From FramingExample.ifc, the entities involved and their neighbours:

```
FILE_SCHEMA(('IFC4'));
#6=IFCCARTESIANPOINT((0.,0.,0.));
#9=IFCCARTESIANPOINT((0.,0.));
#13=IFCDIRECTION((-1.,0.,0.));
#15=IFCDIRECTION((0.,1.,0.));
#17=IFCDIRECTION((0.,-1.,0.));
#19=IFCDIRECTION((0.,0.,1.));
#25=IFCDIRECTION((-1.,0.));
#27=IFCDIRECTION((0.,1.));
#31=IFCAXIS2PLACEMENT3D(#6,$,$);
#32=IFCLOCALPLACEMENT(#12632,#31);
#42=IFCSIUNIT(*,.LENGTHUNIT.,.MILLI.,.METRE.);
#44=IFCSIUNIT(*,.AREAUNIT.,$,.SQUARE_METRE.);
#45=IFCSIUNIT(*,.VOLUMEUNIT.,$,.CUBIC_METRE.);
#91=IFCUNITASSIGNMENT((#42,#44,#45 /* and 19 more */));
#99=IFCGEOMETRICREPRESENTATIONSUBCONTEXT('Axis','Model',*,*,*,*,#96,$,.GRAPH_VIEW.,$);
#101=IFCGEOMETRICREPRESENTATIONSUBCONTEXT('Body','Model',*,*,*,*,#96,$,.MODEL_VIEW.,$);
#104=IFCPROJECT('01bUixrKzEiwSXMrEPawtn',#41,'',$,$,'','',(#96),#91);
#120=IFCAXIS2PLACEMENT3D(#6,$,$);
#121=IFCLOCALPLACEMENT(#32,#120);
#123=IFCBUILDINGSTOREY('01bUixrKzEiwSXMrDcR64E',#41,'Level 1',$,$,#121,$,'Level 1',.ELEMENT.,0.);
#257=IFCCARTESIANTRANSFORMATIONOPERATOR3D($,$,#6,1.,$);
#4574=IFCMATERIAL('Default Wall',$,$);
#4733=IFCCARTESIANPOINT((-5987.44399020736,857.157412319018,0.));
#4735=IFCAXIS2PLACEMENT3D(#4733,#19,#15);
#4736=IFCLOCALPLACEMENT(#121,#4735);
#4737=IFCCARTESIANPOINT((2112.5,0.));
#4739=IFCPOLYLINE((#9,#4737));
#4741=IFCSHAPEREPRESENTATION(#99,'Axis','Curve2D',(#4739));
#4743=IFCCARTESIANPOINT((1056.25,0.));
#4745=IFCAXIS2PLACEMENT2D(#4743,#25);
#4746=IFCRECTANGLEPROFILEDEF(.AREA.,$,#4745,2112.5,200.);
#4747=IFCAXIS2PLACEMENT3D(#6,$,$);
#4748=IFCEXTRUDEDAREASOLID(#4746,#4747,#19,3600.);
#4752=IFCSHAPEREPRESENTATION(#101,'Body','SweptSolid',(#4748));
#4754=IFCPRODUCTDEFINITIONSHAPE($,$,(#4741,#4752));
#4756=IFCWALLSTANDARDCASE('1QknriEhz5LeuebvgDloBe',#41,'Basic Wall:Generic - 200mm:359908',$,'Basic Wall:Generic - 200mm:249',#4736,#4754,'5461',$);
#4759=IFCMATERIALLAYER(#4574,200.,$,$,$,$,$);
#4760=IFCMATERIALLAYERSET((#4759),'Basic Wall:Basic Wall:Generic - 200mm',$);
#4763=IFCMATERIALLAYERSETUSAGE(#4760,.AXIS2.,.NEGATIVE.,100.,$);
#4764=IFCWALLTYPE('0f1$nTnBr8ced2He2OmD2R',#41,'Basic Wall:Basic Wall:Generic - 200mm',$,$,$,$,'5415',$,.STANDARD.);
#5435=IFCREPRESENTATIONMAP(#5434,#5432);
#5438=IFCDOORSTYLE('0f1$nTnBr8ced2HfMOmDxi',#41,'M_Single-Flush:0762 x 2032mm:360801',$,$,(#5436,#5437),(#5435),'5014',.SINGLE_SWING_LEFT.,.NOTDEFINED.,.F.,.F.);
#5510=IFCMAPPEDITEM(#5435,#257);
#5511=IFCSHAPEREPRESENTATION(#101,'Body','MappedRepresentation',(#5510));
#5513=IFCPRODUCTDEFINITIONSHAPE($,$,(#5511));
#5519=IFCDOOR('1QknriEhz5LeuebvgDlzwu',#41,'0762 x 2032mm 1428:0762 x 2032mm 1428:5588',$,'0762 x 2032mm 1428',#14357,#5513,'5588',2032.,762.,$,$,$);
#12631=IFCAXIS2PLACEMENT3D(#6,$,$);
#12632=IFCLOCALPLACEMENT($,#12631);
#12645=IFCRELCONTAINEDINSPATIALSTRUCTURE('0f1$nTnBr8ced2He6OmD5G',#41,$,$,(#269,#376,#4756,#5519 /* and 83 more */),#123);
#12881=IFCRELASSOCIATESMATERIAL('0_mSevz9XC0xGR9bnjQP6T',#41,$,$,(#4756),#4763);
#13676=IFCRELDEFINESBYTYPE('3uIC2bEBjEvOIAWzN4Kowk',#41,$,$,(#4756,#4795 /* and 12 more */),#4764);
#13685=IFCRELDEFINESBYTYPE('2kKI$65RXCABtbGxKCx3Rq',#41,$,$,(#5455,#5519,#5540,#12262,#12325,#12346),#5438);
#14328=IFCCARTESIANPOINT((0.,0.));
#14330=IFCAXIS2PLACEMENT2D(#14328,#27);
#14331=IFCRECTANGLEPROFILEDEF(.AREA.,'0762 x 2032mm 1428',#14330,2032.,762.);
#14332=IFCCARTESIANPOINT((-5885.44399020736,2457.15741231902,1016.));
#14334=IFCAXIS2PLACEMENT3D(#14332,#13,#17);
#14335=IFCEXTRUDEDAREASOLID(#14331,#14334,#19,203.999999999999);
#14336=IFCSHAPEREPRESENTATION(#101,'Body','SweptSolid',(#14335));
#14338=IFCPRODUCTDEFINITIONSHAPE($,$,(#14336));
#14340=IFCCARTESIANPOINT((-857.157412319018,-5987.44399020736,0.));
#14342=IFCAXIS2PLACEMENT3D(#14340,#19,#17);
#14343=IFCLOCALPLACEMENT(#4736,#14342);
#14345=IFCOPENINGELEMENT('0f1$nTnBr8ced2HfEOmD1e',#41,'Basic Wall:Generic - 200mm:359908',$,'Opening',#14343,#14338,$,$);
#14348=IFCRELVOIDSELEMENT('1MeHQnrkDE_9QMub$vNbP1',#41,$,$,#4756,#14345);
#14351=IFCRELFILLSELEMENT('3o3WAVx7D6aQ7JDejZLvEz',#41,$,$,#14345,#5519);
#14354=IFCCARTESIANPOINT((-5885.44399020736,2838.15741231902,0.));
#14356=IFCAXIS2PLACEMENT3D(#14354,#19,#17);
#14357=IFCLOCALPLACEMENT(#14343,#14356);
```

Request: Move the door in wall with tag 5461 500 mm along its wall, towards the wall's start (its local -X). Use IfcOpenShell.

```python
import ifcopenshell
import ifcopenshell.api.geometry
import ifcopenshell.util.placement
import ifcopenshell.util.unit

model = ifcopenshell.open("FramingExample.ifc")
unit_scale = ifcopenshell.util.unit.calculate_unit_scale(model)

door = model.by_guid("1QknriEhz5LeuebvgDlzwu")
opening = door.FillsVoids[0].RelatingOpeningElement
wall = opening.VoidsElements[0].RelatingBuildingElement

wall_matrix = ifcopenshell.util.placement.get_local_placement(wall.ObjectPlacement)
shift = wall_matrix[:3, 0] * -0.5 / unit_scale
before = ifcopenshell.util.placement.get_local_placement(door.ObjectPlacement)[:3, 3].copy()

# The door is placed relative to its opening, so it follows when the opening moves.
matrix = ifcopenshell.util.placement.get_local_placement(opening.ObjectPlacement)
matrix[:3, 3] += shift
ifcopenshell.api.geometry.edit_object_placement(
    model, product=opening, matrix=matrix, is_si=False, should_transform_children=True
)

after = ifcopenshell.util.placement.get_local_placement(door.ObjectPlacement)[:3, 3]
print("door moved by", (after - before).round(3) + 0.0)

model.write("FramingExample_edited.ifc")
```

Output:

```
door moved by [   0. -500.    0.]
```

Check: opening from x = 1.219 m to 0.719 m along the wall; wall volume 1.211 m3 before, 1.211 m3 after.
